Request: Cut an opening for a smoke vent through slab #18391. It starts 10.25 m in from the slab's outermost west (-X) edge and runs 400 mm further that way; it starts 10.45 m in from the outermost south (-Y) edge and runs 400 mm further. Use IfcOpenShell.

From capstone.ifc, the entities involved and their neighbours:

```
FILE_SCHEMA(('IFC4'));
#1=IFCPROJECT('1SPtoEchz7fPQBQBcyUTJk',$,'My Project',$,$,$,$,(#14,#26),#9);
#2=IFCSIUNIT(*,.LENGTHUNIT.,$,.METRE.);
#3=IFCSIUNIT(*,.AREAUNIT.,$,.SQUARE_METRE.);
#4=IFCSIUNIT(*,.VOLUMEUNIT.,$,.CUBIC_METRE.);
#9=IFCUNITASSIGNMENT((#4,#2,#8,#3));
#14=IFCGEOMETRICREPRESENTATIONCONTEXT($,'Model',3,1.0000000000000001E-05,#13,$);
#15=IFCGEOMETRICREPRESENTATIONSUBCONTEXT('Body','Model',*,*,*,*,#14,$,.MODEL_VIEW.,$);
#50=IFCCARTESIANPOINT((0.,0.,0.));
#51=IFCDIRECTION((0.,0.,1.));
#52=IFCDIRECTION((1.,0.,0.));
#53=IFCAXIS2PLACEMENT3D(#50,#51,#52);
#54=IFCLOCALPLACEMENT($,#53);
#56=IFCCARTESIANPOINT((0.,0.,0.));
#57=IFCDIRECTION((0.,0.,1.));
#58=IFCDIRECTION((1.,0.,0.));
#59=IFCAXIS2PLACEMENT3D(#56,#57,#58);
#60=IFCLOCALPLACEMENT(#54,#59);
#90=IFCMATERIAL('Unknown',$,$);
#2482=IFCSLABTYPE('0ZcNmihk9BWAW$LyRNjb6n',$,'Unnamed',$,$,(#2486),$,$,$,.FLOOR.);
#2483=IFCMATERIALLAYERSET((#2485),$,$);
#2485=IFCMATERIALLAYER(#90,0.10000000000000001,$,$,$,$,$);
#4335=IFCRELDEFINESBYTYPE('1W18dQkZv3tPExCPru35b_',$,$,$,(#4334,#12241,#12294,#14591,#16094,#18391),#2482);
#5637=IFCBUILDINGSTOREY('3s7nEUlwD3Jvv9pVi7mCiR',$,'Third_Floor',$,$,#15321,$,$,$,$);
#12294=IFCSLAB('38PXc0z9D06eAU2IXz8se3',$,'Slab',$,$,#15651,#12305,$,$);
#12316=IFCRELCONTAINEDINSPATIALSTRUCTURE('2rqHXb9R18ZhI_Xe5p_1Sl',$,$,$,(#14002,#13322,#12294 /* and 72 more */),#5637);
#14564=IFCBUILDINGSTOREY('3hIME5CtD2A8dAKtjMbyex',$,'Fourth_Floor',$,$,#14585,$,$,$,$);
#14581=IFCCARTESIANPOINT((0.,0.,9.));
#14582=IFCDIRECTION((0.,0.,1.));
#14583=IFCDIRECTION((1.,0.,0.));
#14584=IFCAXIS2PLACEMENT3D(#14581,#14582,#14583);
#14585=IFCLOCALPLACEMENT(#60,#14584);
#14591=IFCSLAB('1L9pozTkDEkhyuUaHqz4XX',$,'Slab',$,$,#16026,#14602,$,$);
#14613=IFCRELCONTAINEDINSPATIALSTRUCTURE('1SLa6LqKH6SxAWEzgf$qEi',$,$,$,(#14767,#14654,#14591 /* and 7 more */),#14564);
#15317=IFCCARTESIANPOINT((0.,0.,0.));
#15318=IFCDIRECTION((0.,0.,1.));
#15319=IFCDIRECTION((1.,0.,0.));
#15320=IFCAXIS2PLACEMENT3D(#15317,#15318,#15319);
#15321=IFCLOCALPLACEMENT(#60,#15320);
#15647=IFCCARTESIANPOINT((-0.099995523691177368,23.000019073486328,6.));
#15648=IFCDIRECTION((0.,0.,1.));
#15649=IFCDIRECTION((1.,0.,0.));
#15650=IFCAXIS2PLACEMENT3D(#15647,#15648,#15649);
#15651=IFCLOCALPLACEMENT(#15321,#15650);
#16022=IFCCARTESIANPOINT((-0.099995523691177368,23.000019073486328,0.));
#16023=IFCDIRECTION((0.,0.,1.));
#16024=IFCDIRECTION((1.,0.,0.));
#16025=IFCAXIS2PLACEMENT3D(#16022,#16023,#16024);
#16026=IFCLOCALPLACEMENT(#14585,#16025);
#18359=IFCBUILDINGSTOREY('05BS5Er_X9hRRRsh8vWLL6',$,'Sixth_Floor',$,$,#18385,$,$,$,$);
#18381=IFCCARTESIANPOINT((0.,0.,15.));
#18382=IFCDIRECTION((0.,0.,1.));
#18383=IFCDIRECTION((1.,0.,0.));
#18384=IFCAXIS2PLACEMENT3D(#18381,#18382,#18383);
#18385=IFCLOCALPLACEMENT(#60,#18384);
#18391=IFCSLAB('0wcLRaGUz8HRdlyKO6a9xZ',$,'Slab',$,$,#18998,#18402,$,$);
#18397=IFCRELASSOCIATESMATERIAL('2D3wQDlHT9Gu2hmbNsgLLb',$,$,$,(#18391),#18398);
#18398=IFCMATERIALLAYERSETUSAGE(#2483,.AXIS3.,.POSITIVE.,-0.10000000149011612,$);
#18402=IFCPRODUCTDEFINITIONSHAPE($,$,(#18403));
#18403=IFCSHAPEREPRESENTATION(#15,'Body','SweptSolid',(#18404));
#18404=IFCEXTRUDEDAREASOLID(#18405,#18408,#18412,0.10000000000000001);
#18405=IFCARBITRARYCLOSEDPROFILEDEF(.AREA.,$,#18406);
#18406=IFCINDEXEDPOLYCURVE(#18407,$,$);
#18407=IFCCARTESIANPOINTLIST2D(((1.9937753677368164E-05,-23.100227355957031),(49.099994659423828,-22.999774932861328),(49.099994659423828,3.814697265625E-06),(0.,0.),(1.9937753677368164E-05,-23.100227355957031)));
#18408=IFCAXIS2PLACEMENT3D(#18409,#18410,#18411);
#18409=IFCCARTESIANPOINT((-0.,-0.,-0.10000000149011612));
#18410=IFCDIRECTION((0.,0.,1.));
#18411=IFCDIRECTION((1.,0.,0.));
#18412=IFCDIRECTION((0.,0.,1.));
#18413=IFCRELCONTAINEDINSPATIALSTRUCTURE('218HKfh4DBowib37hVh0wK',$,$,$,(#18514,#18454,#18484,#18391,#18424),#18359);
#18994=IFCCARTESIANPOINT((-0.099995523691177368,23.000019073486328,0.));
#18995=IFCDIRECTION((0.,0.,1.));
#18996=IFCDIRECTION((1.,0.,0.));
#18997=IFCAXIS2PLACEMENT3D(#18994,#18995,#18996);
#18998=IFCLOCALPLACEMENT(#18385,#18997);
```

```python
import numpy as np
import ifcopenshell
import ifcopenshell.api.feature
import ifcopenshell.api.geometry
import ifcopenshell.api.root
import ifcopenshell.geom
import ifcopenshell.util.placement
import ifcopenshell.util.representation
import ifcopenshell.util.shape
import ifcopenshell.util.unit

model = ifcopenshell.open("capstone.ifc")
unit_scale = ifcopenshell.util.unit.calculate_unit_scale(model)
settings = ifcopenshell.geom.settings()


def volume(element):
    """Net volume in cubic metres, openings subtracted."""
    shape = ifcopenshell.geom.create_shape(settings, element)
    return ifcopenshell.util.shape.get_volume(shape.geometry)


slab = model.by_guid("0wcLRaGUz8HRdlyKO6a9xZ")
before = volume(slab)

# Extent in the slab's own axes, in metres. The edges named are its -X and -Y sides.
slab_shape = ifcopenshell.geom.create_shape(settings, slab)
vertices = ifcopenshell.util.shape.get_vertices(slab_shape.geometry)
x_min, y_min, bottom = vertices.min(axis=0)
top = vertices[:, 2].max()

opening = ifcopenshell.api.root.create_entity(model, ifc_class="IfcOpeningElement", name="Smoke vent opening", predefined_type="OPENING")
context = ifcopenshell.util.representation.get_context(model, "Model", "Body", "MODEL_VIEW")
width, depth = 0.4, 0.4
outline = [(0.0, 0.0), (width, 0.0), (width, depth), (0.0, depth), (0.0, 0.0)]
# Overshoot both faces by 50 mm so the cut is clean.
shape = ifcopenshell.api.geometry.add_slab_representation(
    model, context=context, depth=top - bottom + 0.1, polyline=outline
)
ifcopenshell.api.geometry.assign_representation(model, product=opening, representation=shape)

matrix = ifcopenshell.util.placement.get_local_placement(slab.ObjectPlacement)
matrix[:, 3] = matrix @ np.append(np.array([x_min + 10.25, y_min + 10.45, bottom - 0.05]) / unit_scale, 1.0)
ifcopenshell.api.geometry.edit_object_placement(model, product=opening, matrix=matrix, is_si=False)
ifcopenshell.api.feature.add_feature(model, feature=opening, element=slab)

after = volume(slab)

print(f"slab volume {before:.3f} -> {after:.3f} m3")

model.write("capstone_rev.ifc")
```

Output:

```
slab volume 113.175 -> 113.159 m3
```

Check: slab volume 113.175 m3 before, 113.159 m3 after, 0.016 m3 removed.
